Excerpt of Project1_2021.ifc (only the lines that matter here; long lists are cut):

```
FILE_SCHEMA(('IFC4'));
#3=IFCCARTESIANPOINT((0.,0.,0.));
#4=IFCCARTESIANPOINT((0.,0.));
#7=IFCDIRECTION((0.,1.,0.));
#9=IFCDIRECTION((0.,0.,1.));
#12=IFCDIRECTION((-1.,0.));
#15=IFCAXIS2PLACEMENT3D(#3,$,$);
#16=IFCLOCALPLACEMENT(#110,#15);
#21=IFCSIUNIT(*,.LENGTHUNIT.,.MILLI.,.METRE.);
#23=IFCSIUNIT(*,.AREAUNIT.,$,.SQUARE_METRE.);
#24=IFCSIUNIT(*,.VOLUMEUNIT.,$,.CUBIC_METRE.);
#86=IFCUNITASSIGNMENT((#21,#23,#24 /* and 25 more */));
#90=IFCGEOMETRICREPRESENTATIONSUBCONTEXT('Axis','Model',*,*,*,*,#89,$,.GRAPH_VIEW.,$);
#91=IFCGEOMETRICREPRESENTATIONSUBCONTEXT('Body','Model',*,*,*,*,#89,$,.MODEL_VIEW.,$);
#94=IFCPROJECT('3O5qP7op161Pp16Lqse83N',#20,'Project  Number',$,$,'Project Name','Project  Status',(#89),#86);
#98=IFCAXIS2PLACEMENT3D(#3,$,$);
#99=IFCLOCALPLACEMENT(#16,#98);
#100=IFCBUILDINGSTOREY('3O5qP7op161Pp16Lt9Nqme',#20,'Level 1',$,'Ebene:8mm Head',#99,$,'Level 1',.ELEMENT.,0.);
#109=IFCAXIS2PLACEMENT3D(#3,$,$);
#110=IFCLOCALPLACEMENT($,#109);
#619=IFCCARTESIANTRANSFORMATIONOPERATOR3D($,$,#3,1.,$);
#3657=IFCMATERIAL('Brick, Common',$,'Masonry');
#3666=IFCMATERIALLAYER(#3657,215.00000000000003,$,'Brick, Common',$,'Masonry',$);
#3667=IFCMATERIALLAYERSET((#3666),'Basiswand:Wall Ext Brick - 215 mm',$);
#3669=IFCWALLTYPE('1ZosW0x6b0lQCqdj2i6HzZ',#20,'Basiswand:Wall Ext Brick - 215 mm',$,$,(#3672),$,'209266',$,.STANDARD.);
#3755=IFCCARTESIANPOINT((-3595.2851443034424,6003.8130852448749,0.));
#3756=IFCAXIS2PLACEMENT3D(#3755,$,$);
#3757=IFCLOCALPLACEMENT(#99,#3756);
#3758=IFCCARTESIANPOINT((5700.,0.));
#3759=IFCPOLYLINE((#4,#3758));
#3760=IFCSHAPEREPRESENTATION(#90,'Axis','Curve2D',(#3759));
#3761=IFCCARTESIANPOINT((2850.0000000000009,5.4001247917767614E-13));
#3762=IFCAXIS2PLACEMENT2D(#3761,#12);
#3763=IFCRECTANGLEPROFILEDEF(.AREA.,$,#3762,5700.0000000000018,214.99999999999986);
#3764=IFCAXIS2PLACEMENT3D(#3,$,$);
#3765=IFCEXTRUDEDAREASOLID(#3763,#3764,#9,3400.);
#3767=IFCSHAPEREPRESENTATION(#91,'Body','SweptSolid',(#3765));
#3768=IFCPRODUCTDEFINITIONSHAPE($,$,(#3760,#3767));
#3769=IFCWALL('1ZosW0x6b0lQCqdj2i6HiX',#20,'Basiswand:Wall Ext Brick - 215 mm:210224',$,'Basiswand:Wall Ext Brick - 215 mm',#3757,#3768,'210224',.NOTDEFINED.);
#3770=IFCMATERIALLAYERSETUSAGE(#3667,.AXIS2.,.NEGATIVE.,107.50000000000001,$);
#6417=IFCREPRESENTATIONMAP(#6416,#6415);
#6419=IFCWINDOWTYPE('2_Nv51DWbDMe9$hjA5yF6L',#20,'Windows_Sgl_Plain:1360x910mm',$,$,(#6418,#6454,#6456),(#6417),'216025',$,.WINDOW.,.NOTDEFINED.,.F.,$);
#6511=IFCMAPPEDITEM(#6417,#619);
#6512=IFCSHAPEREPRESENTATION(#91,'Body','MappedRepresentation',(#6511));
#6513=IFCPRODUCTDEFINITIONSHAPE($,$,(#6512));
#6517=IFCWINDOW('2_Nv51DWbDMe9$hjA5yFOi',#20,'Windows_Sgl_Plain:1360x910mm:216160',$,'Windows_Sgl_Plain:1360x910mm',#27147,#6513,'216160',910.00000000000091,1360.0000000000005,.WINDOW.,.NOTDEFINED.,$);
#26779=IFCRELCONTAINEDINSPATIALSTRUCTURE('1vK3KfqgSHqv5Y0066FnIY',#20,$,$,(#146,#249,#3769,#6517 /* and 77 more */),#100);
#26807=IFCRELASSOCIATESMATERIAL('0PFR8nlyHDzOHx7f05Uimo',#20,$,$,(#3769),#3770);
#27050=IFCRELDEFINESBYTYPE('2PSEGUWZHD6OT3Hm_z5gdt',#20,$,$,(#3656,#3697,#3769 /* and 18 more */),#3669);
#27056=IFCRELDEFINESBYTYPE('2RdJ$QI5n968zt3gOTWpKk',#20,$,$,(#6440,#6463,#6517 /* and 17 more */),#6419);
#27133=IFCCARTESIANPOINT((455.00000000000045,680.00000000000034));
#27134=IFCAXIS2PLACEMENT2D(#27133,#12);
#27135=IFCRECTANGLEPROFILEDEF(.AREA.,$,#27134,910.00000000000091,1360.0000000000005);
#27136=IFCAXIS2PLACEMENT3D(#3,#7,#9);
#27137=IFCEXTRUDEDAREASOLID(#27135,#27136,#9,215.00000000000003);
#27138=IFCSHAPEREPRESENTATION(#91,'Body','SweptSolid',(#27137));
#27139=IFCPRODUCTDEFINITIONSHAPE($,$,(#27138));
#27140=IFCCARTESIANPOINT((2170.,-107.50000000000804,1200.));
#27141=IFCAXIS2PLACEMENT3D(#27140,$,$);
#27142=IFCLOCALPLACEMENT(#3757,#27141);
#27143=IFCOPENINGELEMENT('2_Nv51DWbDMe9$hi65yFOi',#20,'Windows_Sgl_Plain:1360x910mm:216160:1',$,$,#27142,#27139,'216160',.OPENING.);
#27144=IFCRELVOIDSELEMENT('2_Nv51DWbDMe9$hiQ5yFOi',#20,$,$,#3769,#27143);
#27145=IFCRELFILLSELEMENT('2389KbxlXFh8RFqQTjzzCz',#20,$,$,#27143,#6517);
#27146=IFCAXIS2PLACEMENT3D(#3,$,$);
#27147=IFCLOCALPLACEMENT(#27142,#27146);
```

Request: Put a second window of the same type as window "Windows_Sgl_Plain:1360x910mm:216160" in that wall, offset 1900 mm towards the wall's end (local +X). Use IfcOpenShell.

```python
import ifcopenshell
import ifcopenshell.api.feature
import ifcopenshell.api.geometry
import ifcopenshell.api.root
import ifcopenshell.geom
import ifcopenshell.util.element
import ifcopenshell.util.placement
import ifcopenshell.util.shape
import ifcopenshell.util.unit

model = ifcopenshell.open("Project1_2021.ifc")
unit_scale = ifcopenshell.util.unit.calculate_unit_scale(model)
settings = ifcopenshell.geom.settings()


def volume(element):
    """Net volume in cubic metres, openings subtracted."""
    shape = ifcopenshell.geom.create_shape(settings, element)
    return ifcopenshell.util.shape.get_volume(shape.geometry)


def reuse_history(source, copy):
    """copy_class also copies each property set's owner history, people and application; keep the originals."""
    for rel in copy.IsDefinedBy:
        if rel.is_a("IfcRelDefinesByProperties") and (history := rel.RelatingPropertyDefinition.OwnerHistory):
            rel.RelatingPropertyDefinition.OwnerHistory = source.OwnerHistory
            ifcopenshell.util.element.remove_deep2(model, history)


window = model.by_id(6517)
opening = window.FillsVoids[0].RelatingOpeningElement
wall = opening.VoidsElements[0].RelatingBuildingElement
before = volume(wall)
shift = ifcopenshell.util.placement.get_local_placement(wall.ObjectPlacement)[:3, 0] * 1.9 / unit_scale

# copy_class copies the void relationship, type, container and properties, but no geometry.
new_opening = ifcopenshell.api.root.copy_class(model, product=opening)
new_opening.Representation = ifcopenshell.util.element.copy_deep(
    model, opening.Representation, exclude=["IfcGeometricRepresentationContext", "IfcRepresentationMap"]
)
new_opening.Name = "Windows_Sgl_Plain:1360x910mm"
new_opening.Tag = None
new_window = ifcopenshell.api.root.copy_class(model, product=window)
new_window.Representation = ifcopenshell.util.element.copy_deep(
    model, window.Representation, exclude=["IfcGeometricRepresentationContext", "IfcRepresentationMap"]
)
new_window.Name = "Windows_Sgl_Plain:1360x910mm"
new_window.Tag = None
reuse_history(window, new_window)
ifcopenshell.api.feature.add_filling(model, opening=new_opening, element=new_window)

for old, new in ((opening, new_opening), (window, new_window)):
    matrix = ifcopenshell.util.placement.get_local_placement(old.ObjectPlacement)
    matrix[:3, 3] += shift
    ifcopenshell.api.geometry.edit_object_placement(model, product=new, matrix=matrix, is_si=False)

after = volume(wall)

print(f"wall volume {before:.3f} -> {after:.3f} m3")

model.write("Project1_2021_v2.ifc")
```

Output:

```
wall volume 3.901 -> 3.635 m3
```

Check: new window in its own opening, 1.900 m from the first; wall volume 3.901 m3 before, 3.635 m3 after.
